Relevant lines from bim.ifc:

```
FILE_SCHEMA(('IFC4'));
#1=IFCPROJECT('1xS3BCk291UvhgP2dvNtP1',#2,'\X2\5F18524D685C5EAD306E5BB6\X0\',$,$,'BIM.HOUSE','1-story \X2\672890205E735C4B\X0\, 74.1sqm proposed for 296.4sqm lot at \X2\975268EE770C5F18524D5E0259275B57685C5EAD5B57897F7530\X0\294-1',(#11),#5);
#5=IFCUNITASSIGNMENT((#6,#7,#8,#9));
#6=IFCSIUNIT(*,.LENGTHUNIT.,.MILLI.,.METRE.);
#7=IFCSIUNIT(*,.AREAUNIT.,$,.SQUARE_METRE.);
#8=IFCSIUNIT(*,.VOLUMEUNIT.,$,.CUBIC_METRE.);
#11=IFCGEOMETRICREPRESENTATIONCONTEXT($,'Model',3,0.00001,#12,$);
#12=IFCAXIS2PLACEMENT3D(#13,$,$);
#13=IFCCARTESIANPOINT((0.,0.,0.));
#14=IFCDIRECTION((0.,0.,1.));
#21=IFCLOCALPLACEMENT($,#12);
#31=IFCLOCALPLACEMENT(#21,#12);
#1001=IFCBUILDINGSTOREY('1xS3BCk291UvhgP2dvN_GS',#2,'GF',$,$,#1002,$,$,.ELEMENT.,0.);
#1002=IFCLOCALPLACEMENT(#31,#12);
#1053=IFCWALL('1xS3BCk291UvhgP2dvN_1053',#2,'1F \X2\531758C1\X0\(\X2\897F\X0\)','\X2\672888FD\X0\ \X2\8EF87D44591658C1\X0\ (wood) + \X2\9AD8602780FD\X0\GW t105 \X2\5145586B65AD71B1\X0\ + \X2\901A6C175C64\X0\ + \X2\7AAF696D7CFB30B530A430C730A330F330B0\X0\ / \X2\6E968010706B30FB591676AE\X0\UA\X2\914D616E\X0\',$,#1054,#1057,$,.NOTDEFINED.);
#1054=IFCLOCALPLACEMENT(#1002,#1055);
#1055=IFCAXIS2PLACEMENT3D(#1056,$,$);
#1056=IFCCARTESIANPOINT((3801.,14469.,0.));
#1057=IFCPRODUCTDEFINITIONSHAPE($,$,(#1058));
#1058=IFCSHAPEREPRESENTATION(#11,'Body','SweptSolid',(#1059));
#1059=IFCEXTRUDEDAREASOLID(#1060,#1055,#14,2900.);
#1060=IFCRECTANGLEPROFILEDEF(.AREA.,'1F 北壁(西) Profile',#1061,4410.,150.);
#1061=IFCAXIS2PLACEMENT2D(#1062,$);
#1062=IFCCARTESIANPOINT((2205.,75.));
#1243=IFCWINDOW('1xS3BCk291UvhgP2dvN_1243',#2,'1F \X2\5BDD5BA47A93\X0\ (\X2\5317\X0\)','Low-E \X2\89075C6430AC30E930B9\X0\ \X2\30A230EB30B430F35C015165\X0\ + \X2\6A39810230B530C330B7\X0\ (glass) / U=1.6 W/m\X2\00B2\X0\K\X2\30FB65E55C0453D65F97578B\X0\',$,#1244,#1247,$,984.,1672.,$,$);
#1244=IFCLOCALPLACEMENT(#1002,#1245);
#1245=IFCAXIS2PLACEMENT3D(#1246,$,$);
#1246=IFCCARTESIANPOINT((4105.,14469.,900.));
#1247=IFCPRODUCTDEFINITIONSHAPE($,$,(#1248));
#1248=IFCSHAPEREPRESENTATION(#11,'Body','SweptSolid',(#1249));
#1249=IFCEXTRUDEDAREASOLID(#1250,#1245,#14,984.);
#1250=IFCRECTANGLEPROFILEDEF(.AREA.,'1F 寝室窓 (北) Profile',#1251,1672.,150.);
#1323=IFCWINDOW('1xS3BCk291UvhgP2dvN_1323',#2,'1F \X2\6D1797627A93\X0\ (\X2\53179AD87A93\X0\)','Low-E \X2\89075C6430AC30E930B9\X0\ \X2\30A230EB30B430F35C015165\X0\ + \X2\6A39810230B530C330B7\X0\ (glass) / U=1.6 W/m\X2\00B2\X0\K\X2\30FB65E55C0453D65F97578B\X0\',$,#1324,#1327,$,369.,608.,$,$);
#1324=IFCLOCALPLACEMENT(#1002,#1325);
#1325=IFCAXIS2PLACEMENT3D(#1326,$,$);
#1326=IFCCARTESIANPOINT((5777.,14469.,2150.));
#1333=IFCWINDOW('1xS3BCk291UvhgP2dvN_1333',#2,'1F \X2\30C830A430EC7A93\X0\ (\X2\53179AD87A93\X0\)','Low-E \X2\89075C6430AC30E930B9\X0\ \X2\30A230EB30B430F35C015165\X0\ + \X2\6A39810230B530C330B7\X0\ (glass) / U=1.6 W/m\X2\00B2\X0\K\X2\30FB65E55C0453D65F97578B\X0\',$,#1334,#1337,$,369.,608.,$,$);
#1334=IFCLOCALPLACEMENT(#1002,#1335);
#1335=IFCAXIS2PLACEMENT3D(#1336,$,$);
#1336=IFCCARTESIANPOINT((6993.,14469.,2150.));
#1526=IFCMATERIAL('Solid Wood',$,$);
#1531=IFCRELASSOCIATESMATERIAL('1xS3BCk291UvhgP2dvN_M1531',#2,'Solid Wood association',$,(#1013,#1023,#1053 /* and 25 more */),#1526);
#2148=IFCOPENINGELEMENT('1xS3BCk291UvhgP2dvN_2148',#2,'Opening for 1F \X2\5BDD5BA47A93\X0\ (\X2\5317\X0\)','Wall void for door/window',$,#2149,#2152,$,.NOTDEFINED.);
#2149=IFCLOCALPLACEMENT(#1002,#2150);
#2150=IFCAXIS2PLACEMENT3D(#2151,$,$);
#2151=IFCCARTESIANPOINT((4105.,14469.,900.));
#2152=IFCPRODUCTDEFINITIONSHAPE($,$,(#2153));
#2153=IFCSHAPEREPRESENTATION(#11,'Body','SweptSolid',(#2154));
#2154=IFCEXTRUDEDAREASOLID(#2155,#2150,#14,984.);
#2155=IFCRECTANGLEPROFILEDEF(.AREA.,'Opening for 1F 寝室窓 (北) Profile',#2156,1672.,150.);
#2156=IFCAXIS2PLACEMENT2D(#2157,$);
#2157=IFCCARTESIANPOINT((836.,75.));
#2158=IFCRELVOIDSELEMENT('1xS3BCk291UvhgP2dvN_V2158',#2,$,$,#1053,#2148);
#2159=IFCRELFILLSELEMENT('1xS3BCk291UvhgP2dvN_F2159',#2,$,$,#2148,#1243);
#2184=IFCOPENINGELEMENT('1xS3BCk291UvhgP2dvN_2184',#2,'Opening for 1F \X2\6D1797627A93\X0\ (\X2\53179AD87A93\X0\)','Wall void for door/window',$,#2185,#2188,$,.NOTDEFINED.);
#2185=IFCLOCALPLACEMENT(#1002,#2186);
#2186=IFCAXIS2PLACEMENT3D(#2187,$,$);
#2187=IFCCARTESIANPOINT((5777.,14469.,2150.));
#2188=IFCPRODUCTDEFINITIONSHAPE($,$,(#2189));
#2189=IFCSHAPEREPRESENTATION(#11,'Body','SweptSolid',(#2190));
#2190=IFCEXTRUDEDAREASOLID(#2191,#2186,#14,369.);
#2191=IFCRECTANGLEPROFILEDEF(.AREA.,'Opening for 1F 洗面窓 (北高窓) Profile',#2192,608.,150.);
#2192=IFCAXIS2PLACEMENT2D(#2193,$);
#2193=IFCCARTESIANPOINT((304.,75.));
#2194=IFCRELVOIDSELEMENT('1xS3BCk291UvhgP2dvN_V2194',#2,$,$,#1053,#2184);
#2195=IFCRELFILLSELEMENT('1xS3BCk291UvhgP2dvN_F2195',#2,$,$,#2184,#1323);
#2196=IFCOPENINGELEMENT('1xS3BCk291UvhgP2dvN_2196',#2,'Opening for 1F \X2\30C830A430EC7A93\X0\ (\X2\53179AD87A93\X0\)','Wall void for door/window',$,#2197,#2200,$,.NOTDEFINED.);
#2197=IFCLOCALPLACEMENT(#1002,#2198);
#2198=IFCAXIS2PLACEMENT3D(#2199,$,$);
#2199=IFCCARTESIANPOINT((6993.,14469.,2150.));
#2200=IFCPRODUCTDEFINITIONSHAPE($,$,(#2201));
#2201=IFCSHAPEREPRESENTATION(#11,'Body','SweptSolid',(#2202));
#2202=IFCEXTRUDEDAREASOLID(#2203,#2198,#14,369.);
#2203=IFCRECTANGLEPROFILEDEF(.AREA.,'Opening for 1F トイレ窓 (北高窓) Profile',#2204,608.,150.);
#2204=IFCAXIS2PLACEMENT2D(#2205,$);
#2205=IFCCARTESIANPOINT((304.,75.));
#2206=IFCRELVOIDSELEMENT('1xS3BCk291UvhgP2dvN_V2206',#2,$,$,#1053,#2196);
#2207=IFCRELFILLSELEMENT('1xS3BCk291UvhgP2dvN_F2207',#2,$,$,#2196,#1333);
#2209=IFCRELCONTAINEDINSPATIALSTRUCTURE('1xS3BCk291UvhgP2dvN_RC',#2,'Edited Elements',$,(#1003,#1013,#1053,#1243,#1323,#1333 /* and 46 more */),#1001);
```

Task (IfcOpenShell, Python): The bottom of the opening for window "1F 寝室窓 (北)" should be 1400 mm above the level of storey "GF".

```python
import numpy as np
import ifcopenshell
import ifcopenshell.api.geometry
import ifcopenshell.geom
import ifcopenshell.util.element
import ifcopenshell.util.placement
import ifcopenshell.util.shape
import ifcopenshell.util.unit

model = ifcopenshell.open("bim.ifc")
unit_scale = ifcopenshell.util.unit.calculate_unit_scale(model)

window = model.by_guid("1xS3BCk291UvhgP2dvN_1243")
opening = window.FillsVoids[0].RelatingOpeningElement
storey = ifcopenshell.util.element.get_container(window, ifc_class="IfcBuildingStorey")
level = ifcopenshell.util.placement.get_local_placement(storey.ObjectPlacement)[2, 3]

# The opening's origin need not be at the sill, so measure its lowest point.
shape = ifcopenshell.geom.create_shape(ifcopenshell.geom.settings(), opening)
bottom = ifcopenshell.util.shape.get_shape_bottom_elevation(shape, shape.geometry) / unit_scale
dz = level + 1.4 / unit_scale - bottom

shift = np.array([0.0, 0.0, dz])
# The window is not placed relative to its opening, so move both.
for product in (opening, window):
    matrix = ifcopenshell.util.placement.get_local_placement(product.ObjectPlacement)
    matrix[:3, 3] += shift
    ifcopenshell.api.geometry.edit_object_placement(model, product=product, matrix=matrix, is_si=False)

print(f"moved by {dz * unit_scale:+.3f} m")

model.write("bim_edited.ifc")
```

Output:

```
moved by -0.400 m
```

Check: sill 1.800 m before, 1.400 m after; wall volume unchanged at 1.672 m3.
